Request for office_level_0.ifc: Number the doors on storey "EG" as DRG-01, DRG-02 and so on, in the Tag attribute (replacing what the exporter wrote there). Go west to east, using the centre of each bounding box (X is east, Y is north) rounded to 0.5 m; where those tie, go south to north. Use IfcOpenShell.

First a look at what the model holds.

```python
import ifcopenshell
import ifcopenshell.util.element
import ifcopenshell.util.placement

model = ifcopenshell.open("office_level_0.ifc")
print(model.schema)
storey = next(s for s in model.by_type("IfcBuildingStorey") if s.Name == "EG")
doors = [e for e in ifcopenshell.util.element.get_decomposition(storey) if e.is_a("IfcDoor")]
for e in sorted(doors, key=lambda e: e.id()):
    origin = ifcopenshell.util.placement.get_local_placement(e.ObjectPlacement)[:3, 3]
    print(e.id(), e.Tag, e.Name, origin.round(2) + 0.0, sep=" | ")
```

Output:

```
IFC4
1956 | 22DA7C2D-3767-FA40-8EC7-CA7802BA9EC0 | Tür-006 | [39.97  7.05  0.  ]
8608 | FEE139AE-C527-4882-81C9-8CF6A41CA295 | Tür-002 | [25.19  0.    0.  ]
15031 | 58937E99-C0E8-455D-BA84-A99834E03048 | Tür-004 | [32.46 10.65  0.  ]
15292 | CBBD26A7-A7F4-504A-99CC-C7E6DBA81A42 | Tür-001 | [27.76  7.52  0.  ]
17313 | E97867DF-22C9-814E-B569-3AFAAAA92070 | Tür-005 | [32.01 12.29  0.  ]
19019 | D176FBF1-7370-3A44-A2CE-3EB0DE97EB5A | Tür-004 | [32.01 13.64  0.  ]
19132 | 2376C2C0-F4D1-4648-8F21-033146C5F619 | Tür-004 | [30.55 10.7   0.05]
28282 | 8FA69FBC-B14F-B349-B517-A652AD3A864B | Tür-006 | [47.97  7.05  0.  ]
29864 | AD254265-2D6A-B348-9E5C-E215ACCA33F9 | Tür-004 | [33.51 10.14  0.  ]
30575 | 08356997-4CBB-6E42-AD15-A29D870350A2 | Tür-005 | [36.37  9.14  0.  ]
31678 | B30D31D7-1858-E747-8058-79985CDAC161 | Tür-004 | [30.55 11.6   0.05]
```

```python
import ifcopenshell
import ifcopenshell.geom
import ifcopenshell.util.element
import ifcopenshell.util.shape

model = ifcopenshell.open("office_level_0.ifc")
settings = ifcopenshell.geom.settings()
settings.set("use-world-coords", True)


def centre(element):
    shape = ifcopenshell.geom.create_shape(settings, element)
    return ifcopenshell.util.shape.get_bbox_centroid(shape.geometry)


storey = next(s for s in model.by_type("IfcBuildingStorey") if s.Name == "EG")
doors = [e for e in ifcopenshell.util.element.get_decomposition(storey) if e.is_a("IfcDoor")]

# Insertion points can sit at a corner or the storey origin, so sort by the geometry (in metres).
centres = {e: centre(e) for e in doors}
doors.sort(key=lambda e: (round(centres[e][0] / 0.5), centres[e][1]))

for i, e in enumerate(doors, start=1):
    number = f"DRG-{i:02d}"
    e.Tag = number
    print(e.id(), number)

model.write("office_level_0-out.ifc")
```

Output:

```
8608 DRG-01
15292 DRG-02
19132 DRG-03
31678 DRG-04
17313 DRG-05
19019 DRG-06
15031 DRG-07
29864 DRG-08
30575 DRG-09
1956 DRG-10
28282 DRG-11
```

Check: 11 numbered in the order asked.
